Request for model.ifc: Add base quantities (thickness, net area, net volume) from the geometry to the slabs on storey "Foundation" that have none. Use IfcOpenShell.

First a look at what the model holds.

```python
import ifcopenshell
import ifcopenshell.util.element
import ifcopenshell.util.unit

model = ifcopenshell.open("model.ifc")
print(model.schema)
for unit_type in ("LENGTHUNIT", "AREAUNIT", "VOLUMEUNIT"):
    print(unit_type, ifcopenshell.util.unit.calculate_unit_scale(model, unit_type))
storey = next(s for s in model.by_type("IfcBuildingStorey") if s.Name == "Foundation")
slabs = [e for e in ifcopenshell.util.element.get_decomposition(storey) if e.is_a("IfcSlab")]
for e in sorted(slabs, key=lambda e: e.id()):
    print(e.id(), e.is_a(), e.Name, list(ifcopenshell.util.element.get_psets(e, qtos_only=True)), sep=" | ")
```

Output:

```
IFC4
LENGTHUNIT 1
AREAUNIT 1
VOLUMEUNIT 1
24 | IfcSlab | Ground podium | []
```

```python
import ifcopenshell
import ifcopenshell.api.pset
import ifcopenshell.geom
import ifcopenshell.util.element
import ifcopenshell.util.shape
import ifcopenshell.util.unit

model = ifcopenshell.open("model.ifc")
unit_scale = ifcopenshell.util.unit.calculate_unit_scale(model)
area_scale = ifcopenshell.util.unit.calculate_unit_scale(model, "AREAUNIT")
volume_scale = ifcopenshell.util.unit.calculate_unit_scale(model, "VOLUMEUNIT")
settings = ifcopenshell.geom.settings()

storey = next(s for s in model.by_type("IfcBuildingStorey") if s.Name == "Foundation")
slabs = [e for e in ifcopenshell.util.element.get_decomposition(storey) if e.is_a("IfcSlab")]

for e in sorted(slabs, key=lambda e: e.id()):
    if ifcopenshell.util.element.get_psets(e, qtos_only=True, should_inherit=False):
        continue
    # Geometry comes back in metres, in the element's own axes.
    shape = ifcopenshell.geom.create_shape(settings, e)
    values = {
        "Width": ifcopenshell.util.shape.get_z(shape.geometry) / unit_scale,
        "NetArea": ifcopenshell.util.shape.get_footprint_area(shape.geometry) / area_scale,
        "NetVolume": ifcopenshell.util.shape.get_volume(shape.geometry) / volume_scale,
    }
    qto = ifcopenshell.api.pset.add_qto(model, product=e, name="Qto_SlabBaseQuantities")
    ifcopenshell.api.pset.edit_qto(model, qto=qto, properties=values)
    print(e.id(), {k: round(v, 3) for k, v in values.items()})

model.write("model_updated.ifc")
```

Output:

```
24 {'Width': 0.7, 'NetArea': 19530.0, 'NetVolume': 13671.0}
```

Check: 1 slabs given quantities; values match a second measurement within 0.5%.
